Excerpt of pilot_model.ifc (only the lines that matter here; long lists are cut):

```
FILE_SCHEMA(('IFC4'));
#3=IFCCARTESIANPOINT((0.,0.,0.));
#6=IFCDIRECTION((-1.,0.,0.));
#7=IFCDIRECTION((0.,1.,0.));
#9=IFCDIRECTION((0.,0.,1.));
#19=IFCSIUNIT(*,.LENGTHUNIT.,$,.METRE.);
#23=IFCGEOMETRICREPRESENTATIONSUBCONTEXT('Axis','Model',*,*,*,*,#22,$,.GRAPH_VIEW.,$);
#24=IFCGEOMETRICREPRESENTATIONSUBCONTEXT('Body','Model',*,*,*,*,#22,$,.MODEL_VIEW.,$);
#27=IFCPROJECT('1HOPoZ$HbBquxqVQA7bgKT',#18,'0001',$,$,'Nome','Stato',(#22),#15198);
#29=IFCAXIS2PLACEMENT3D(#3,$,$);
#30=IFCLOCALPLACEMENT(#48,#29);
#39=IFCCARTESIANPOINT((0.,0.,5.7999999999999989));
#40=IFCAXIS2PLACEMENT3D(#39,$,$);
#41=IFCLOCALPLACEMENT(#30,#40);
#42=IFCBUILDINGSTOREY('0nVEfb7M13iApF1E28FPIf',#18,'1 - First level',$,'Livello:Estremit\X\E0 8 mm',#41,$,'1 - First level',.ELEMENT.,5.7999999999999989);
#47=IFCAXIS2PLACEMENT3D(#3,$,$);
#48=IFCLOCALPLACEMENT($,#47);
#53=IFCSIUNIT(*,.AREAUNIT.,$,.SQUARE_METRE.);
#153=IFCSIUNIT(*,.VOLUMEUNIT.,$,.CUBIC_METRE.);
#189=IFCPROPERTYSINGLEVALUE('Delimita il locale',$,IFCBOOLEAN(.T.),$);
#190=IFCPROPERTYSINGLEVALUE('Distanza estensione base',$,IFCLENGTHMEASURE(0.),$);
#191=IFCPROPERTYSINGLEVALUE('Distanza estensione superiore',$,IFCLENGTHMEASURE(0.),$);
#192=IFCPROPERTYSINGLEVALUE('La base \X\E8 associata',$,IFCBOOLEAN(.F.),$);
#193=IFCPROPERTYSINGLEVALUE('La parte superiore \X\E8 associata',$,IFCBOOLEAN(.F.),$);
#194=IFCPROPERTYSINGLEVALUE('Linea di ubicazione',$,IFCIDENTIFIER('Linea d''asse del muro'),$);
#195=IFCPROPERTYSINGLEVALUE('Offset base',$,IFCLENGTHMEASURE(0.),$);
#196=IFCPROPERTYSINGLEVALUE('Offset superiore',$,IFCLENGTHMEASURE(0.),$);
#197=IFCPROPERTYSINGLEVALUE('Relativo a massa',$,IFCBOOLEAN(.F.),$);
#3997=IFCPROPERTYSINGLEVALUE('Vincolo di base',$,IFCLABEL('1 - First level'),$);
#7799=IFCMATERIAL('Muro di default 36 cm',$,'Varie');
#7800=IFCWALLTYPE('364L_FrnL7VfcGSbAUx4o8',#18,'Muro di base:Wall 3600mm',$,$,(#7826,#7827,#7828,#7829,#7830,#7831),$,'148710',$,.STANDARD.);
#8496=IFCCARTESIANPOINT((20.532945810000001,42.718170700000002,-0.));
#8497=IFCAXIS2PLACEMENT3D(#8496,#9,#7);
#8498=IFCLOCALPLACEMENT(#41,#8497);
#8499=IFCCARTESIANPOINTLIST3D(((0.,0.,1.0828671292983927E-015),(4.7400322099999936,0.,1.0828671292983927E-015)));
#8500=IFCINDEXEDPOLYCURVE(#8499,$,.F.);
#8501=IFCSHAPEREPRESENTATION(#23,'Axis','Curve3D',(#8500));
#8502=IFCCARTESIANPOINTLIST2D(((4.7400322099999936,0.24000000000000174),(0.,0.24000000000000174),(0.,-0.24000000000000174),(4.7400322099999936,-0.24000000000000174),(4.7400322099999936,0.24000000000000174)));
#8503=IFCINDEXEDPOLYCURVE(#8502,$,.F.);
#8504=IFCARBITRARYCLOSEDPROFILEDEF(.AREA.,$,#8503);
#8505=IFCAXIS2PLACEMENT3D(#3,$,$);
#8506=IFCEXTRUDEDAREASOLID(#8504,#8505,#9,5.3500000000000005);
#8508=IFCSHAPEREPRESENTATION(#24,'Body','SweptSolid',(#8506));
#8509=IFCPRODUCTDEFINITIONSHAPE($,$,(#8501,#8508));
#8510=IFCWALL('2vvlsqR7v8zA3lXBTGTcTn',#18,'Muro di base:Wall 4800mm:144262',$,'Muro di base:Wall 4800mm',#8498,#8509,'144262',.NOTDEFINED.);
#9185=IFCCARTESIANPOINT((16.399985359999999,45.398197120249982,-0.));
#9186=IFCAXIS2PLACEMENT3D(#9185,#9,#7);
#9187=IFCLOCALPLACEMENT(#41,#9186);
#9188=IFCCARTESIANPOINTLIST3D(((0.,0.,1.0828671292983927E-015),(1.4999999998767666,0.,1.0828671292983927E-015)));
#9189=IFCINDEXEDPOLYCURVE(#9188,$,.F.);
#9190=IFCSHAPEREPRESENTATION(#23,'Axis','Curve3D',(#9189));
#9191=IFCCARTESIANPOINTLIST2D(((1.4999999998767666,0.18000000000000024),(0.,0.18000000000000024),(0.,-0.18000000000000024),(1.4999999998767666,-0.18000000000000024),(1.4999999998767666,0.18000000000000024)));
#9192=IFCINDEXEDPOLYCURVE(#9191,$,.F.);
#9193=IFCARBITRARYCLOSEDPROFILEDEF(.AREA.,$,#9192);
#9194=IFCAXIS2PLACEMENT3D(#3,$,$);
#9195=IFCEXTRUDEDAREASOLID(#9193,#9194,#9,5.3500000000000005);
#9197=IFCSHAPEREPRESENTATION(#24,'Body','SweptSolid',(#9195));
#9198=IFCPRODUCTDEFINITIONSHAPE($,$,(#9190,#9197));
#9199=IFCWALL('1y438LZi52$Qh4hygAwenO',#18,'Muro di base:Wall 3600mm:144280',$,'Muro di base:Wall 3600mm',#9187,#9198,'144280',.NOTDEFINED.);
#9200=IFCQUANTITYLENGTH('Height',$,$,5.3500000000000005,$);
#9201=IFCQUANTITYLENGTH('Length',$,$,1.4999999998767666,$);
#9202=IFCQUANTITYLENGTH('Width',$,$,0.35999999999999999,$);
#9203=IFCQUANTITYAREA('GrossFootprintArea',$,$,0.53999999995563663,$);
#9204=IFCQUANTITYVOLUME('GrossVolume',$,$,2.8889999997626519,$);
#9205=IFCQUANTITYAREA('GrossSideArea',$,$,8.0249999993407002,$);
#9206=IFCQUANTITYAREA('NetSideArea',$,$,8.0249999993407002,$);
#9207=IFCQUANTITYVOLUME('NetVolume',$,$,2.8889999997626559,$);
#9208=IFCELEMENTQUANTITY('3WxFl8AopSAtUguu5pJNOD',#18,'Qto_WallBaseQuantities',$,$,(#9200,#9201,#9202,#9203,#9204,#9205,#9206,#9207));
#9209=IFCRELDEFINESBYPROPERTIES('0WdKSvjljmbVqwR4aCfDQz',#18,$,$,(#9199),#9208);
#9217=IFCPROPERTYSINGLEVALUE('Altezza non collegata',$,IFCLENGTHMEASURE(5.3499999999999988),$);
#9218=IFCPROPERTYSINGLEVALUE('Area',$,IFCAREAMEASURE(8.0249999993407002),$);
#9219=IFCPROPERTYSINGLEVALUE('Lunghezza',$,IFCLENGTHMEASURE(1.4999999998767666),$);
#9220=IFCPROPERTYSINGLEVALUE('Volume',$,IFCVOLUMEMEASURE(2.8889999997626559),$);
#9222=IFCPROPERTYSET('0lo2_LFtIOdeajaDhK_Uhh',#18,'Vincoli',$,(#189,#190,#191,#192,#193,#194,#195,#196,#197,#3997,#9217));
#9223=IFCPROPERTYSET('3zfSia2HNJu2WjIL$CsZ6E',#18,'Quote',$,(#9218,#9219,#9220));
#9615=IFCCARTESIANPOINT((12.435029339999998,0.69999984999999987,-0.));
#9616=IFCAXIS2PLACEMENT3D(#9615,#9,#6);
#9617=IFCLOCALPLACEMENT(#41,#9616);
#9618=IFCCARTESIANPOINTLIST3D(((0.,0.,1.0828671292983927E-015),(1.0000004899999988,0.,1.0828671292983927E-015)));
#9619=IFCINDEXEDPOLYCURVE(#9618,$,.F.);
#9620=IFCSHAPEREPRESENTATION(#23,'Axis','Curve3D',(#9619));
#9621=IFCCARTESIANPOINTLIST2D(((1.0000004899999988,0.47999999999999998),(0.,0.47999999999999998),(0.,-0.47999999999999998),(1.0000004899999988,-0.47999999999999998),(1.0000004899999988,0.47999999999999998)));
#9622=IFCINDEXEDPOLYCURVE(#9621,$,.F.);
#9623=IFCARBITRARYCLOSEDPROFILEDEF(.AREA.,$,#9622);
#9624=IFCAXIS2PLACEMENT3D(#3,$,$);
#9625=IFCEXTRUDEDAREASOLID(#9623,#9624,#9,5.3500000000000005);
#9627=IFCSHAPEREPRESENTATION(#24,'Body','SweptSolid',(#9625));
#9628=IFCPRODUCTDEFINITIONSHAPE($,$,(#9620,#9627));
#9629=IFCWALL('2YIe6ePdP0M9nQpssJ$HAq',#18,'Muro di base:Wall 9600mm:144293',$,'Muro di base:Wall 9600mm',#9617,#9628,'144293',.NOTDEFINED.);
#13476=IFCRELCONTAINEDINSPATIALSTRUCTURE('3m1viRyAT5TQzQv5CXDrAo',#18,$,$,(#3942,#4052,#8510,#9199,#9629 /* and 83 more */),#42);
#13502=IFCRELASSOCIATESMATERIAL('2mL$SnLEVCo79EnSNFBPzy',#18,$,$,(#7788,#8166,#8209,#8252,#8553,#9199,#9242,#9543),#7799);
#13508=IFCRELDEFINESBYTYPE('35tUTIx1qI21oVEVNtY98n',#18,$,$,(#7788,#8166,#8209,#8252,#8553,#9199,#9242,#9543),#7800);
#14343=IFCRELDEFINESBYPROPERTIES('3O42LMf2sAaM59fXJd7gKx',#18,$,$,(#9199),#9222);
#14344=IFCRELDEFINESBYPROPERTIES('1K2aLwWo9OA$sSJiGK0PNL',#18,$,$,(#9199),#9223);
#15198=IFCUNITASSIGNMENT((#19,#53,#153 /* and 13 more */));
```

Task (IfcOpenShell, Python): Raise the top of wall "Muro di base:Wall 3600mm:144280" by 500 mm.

```python
import ifcopenshell
import ifcopenshell.api.pset
import ifcopenshell.geom
import ifcopenshell.util.element
import ifcopenshell.util.representation
import ifcopenshell.util.shape
import ifcopenshell.util.unit

model = ifcopenshell.open("pilot_model.ifc")
unit_scale = ifcopenshell.util.unit.calculate_unit_scale(model)
area_scale = ifcopenshell.util.unit.calculate_unit_scale(model, "AREAUNIT")
volume_scale = ifcopenshell.util.unit.calculate_unit_scale(model, "VOLUMEUNIT")
settings = ifcopenshell.geom.settings()


def volume(element):
    """Net volume in cubic metres, openings subtracted."""
    shape = ifcopenshell.geom.create_shape(settings, element)
    return ifcopenshell.util.shape.get_volume(shape.geometry)


wall = model.by_guid("1y438LZi52$Qh4hygAwenO")
before = volume(wall)

body = ifcopenshell.util.representation.get_representation(wall, "Model", "Body")
solid = body.Items[0]
old_height = solid.Depth
solid.Depth += 0.5 / unit_scale
after = volume(wall)
thickness = 0.36  # wall thickness in metres

# Update the stored height, areas and volumes.
qto = model.by_id(ifcopenshell.util.element.get_pset(wall, "Qto_WallBaseQuantities", should_inherit=False)["id"])
ifcopenshell.api.pset.edit_qto(model, qto=qto, properties={
    "Height": solid.Depth,
    "GrossVolume": ifcopenshell.util.element.get_pset(wall, "Qto_WallBaseQuantities", "GrossVolume") * solid.Depth / old_height,
    "GrossSideArea": ifcopenshell.util.element.get_pset(wall, "Qto_WallBaseQuantities", "GrossSideArea") * solid.Depth / old_height,
    "NetSideArea": after / thickness / area_scale,
    "NetVolume": after / volume_scale,
})
pset = model.by_id(ifcopenshell.util.element.get_pset(wall, "Vincoli", should_inherit=False)["id"])
ifcopenshell.api.pset.edit_pset(model, pset=pset, properties={
    "Altezza non collegata": model.create_entity("IfcLengthMeasure", solid.Depth),
})
pset = model.by_id(ifcopenshell.util.element.get_pset(wall, "Quote", should_inherit=False)["id"])
ifcopenshell.api.pset.edit_pset(model, pset=pset, properties={
    "Area": model.create_entity("IfcAreaMeasure", after / thickness / area_scale),
    "Volume": model.create_entity("IfcVolumeMeasure", after / volume_scale),
})

print(f"height {old_height:g} -> {solid.Depth:g}, volume {before:.3f} -> {after:.3f} m3")

model.write("pilot_model_v2.ifc")
```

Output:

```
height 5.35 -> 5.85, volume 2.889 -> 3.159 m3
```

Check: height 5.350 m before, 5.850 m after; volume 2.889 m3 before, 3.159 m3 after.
